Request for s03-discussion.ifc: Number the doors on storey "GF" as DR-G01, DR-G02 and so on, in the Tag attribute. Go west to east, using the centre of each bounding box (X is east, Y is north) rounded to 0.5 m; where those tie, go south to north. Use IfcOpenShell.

First a look at what the model holds.

```python
import ifcopenshell
import ifcopenshell.util.element
import ifcopenshell.util.placement

model = ifcopenshell.open("s03-discussion.ifc")
print(model.schema)
storey = next(s for s in model.by_type("IfcBuildingStorey") if s.Name == "GF")
doors = [e for e in ifcopenshell.util.element.get_decomposition(storey) if e.is_a("IfcDoor")]
for e in sorted(doors, key=lambda e: e.id()):
    origin = ifcopenshell.util.placement.get_local_placement(e.ObjectPlacement)[:3, 3]
    print(e.id(), e.Tag, e.Name, origin.round(2) + 0.0, sep=" | ")
```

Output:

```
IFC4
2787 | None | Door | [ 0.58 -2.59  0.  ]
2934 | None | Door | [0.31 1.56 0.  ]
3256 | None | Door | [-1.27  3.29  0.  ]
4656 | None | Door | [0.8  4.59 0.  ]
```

```python
import ifcopenshell
import ifcopenshell.geom
import ifcopenshell.util.element
import ifcopenshell.util.shape

model = ifcopenshell.open("s03-discussion.ifc")
settings = ifcopenshell.geom.settings()
settings.set("use-world-coords", True)


def centre(element):
    shape = ifcopenshell.geom.create_shape(settings, element)
    return ifcopenshell.util.shape.get_bbox_centroid(shape.geometry)


storey = next(s for s in model.by_type("IfcBuildingStorey") if s.Name == "GF")
doors = [e for e in ifcopenshell.util.element.get_decomposition(storey) if e.is_a("IfcDoor")]

# Insertion points can sit at a corner or the storey origin, so sort by the geometry (in metres).
centres = {e: centre(e) for e in doors}
doors.sort(key=lambda e: (round(centres[e][0] / 0.5), centres[e][1]))

for i, e in enumerate(doors, start=1):
    number = f"DR-G{i:02d}"
    e.Tag = number
    print(e.id(), number)

model.write("s03-discussion-out.ifc")
```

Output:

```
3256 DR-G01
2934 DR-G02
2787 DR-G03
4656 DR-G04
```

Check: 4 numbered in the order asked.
